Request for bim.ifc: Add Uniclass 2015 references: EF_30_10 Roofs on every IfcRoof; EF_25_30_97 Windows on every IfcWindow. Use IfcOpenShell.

First a look at what the model holds.

```python
import ifcopenshell

model = ifcopenshell.open("bim.ifc")
print(model.schema)
print("classifications:", [c.Name for c in model.by_type("IfcClassification")])
for ifc_class in ("IfcDoor", "IfcRoof", "IfcStair", "IfcWall", "IfcWindow"):
    print(ifc_class, len(model.by_type(ifc_class)))
```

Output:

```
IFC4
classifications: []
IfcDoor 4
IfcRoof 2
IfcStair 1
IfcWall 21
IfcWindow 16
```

```python
import ifcopenshell
import ifcopenshell.api.classification

model = ifcopenshell.open("bim.ifc")

system = ifcopenshell.api.classification.add_classification(model, classification="Uniclass 2015")

codes = {
    "IfcRoof": ("EF_30_10", "Roofs"),
    "IfcWindow": ("EF_25_30_97", "Windows"),
}
for ifc_class, (code, name) in codes.items():
    products = model.by_type(ifc_class)
    ifcopenshell.api.classification.add_reference(
        model, products=products, classification=system, identification=code, name=name
    )
    print(code, len(products))

model.write("bim_updated.ifc")
```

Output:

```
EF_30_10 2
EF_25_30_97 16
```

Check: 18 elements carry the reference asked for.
